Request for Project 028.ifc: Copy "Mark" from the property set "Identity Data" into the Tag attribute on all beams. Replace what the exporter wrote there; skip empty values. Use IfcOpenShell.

First a look at what the model holds.

```python
import ifcopenshell
import ifcopenshell.util.element

model = ifcopenshell.open("Project 028.ifc")
print(model.schema)
beams = model.by_type("IfcBeam")
print(len(beams), "beams")
for e in beams[:8]:
    source = ifcopenshell.util.element.get_pset(e, "Identity Data", "Mark")
    target = e.Tag
    print(e.id(), repr(source), repr(target), sep=" | ")
```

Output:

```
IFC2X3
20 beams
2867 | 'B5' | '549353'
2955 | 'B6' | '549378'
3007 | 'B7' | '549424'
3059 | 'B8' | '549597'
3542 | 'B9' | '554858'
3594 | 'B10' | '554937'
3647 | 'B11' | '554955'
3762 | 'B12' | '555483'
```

```python
import ifcopenshell
import ifcopenshell.util.element

model = ifcopenshell.open("Project 028.ifc")

count = 0
for e in model.by_type("IfcBeam"):
    value = ifcopenshell.util.element.get_pset(e, "Identity Data", "Mark")
    current = e.Tag
    if not value or not value.strip() or current == value:
        continue
    e.Tag = value
    count += 1

print(count, "beams updated")

model.write("Project 028_v2.ifc")
```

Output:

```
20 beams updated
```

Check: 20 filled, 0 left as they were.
